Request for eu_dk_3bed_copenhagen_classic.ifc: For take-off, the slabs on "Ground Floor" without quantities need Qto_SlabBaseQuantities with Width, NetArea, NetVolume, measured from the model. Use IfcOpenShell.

First a look at what the model holds.

```python
import ifcopenshell
import ifcopenshell.util.element
import ifcopenshell.util.unit

model = ifcopenshell.open("eu_dk_3bed_copenhagen_classic.ifc")
print(model.schema)
for unit_type in ("LENGTHUNIT", "AREAUNIT", "VOLUMEUNIT"):
    print(unit_type, ifcopenshell.util.unit.calculate_unit_scale(model, unit_type))
storey = next(s for s in model.by_type("IfcBuildingStorey") if s.Name == "Ground Floor")
slabs = [e for e in ifcopenshell.util.element.get_decomposition(storey) if e.is_a("IfcSlab")]
for e in sorted(slabs, key=lambda e: e.id()):
    print(e.id(), e.is_a(), e.Name, list(ifcopenshell.util.element.get_psets(e, qtos_only=True)), sep=" | ")
```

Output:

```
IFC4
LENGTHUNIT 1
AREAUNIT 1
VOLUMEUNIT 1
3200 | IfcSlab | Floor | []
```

```python
import ifcopenshell
import ifcopenshell.api.pset
import ifcopenshell.geom
import ifcopenshell.util.element
import ifcopenshell.util.shape
import ifcopenshell.util.unit

model = ifcopenshell.open("eu_dk_3bed_copenhagen_classic.ifc")
unit_scale = ifcopenshell.util.unit.calculate_unit_scale(model)
area_scale = ifcopenshell.util.unit.calculate_unit_scale(model, "AREAUNIT")
volume_scale = ifcopenshell.util.unit.calculate_unit_scale(model, "VOLUMEUNIT")
settings = ifcopenshell.geom.settings()

storey = next(s for s in model.by_type("IfcBuildingStorey") if s.Name == "Ground Floor")
slabs = [e for e in ifcopenshell.util.element.get_decomposition(storey) if e.is_a("IfcSlab")]

for e in sorted(slabs, key=lambda e: e.id()):
    if ifcopenshell.util.element.get_psets(e, qtos_only=True, should_inherit=False):
        continue
    # Geometry comes back in metres, in the element's own axes.
    shape = ifcopenshell.geom.create_shape(settings, e)
    values = {
        "Width": ifcopenshell.util.shape.get_z(shape.geometry) / unit_scale,
        "NetArea": ifcopenshell.util.shape.get_footprint_area(shape.geometry) / area_scale,
        "NetVolume": ifcopenshell.util.shape.get_volume(shape.geometry) / volume_scale,
    }
    qto = ifcopenshell.api.pset.add_qto(model, product=e, name="Qto_SlabBaseQuantities")
    ifcopenshell.api.pset.edit_qto(model, qto=qto, properties=values)
    print(e.id(), {k: round(v, 3) for k, v in values.items()})

model.write("eu_dk_3bed_copenhagen_classic_edited.ifc")
```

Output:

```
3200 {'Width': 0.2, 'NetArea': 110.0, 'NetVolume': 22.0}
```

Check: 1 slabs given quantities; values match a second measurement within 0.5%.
